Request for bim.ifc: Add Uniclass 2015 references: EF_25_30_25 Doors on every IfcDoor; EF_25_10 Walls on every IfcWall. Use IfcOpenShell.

First a look at what the model holds.

```python
import ifcopenshell

model = ifcopenshell.open("bim.ifc")
print(model.schema)
print("classifications:", [c.Name for c in model.by_type("IfcClassification")])
for ifc_class in ("IfcDoor", "IfcRoof", "IfcStair", "IfcWall", "IfcWindow"):
    print(ifc_class, len(model.by_type(ifc_class)))
```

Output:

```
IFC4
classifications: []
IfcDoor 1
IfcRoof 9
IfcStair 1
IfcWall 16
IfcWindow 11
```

```python
import ifcopenshell
import ifcopenshell.api.classification

model = ifcopenshell.open("bim.ifc")

system = ifcopenshell.api.classification.add_classification(model, classification="Uniclass 2015")

codes = {
    "IfcDoor": ("EF_25_30_25", "Doors"),
    "IfcWall": ("EF_25_10", "Walls"),
}
for ifc_class, (code, name) in codes.items():
    products = model.by_type(ifc_class)
    ifcopenshell.api.classification.add_reference(
        model, products=products, classification=system, identification=code, name=name
    )
    print(code, len(products))

model.write("bim_rev.ifc")
```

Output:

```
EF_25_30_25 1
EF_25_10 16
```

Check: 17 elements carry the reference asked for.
